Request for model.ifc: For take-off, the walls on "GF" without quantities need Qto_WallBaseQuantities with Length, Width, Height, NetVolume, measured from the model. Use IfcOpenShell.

First a look at what the model holds.

```python
import ifcopenshell
import ifcopenshell.util.element
import ifcopenshell.util.unit

model = ifcopenshell.open("model.ifc")
print(model.schema)
for unit_type in ("LENGTHUNIT", "AREAUNIT", "VOLUMEUNIT"):
    print(unit_type, ifcopenshell.util.unit.calculate_unit_scale(model, unit_type))
storey = next(s for s in model.by_type("IfcBuildingStorey") if s.Name == "GF")
walls = [e for e in ifcopenshell.util.element.get_decomposition(storey) if e.is_a("IfcWall")]
for e in sorted(walls, key=lambda e: e.id()):
    print(e.id(), e.is_a(), e.Name, list(ifcopenshell.util.element.get_psets(e, qtos_only=True)), sep=" | ")
```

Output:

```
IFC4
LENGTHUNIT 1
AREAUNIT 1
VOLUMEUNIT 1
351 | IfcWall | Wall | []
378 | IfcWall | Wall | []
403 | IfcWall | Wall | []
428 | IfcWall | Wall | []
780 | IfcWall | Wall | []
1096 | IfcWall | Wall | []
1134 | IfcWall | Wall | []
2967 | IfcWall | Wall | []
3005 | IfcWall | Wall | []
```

```python
import ifcopenshell
import ifcopenshell.api.pset
import ifcopenshell.geom
import ifcopenshell.util.element
import ifcopenshell.util.shape
import ifcopenshell.util.unit

model = ifcopenshell.open("model.ifc")
unit_scale = ifcopenshell.util.unit.calculate_unit_scale(model)
volume_scale = ifcopenshell.util.unit.calculate_unit_scale(model, "VOLUMEUNIT")
settings = ifcopenshell.geom.settings()

storey = next(s for s in model.by_type("IfcBuildingStorey") if s.Name == "GF")
walls = [e for e in ifcopenshell.util.element.get_decomposition(storey) if e.is_a("IfcWall")]

for e in sorted(walls, key=lambda e: e.id()):
    if ifcopenshell.util.element.get_psets(e, qtos_only=True, should_inherit=False):
        continue
    # Geometry comes back in metres, in the element's own axes.
    shape = ifcopenshell.geom.create_shape(settings, e)
    values = {
        "Length": ifcopenshell.util.shape.get_x(shape.geometry) / unit_scale,
        "Width": ifcopenshell.util.shape.get_y(shape.geometry) / unit_scale,
        "Height": ifcopenshell.util.shape.get_z(shape.geometry) / unit_scale,
        "NetVolume": ifcopenshell.util.shape.get_volume(shape.geometry) / volume_scale,
    }
    qto = ifcopenshell.api.pset.add_qto(model, product=e, name="Qto_WallBaseQuantities")
    ifcopenshell.api.pset.edit_qto(model, qto=qto, properties=values)
    print(e.id(), {k: round(v, 3) for k, v in values.items()})

model.write("model_rev.ifc")
```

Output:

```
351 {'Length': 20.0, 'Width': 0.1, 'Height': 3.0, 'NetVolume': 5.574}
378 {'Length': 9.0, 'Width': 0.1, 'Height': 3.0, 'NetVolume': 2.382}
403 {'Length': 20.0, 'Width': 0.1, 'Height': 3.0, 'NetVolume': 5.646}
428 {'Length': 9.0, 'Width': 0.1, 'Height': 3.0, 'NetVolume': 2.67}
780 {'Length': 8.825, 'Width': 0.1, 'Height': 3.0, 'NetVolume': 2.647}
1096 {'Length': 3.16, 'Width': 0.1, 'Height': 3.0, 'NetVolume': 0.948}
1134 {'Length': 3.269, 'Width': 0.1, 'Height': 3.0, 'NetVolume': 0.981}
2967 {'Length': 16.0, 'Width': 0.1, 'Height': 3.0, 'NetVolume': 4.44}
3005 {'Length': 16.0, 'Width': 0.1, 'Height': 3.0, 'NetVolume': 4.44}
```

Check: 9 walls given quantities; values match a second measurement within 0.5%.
